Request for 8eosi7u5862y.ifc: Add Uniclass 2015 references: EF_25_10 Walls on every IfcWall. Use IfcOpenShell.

First a look at what the model holds.

```python
import ifcopenshell

model = ifcopenshell.open("8eosi7u5862y.ifc")
print(model.schema)
print("classifications:", [c.Name for c in model.by_type("IfcClassification")])
for ifc_class in ("IfcDoor", "IfcRoof", "IfcStair", "IfcWall", "IfcWindow"):
    print(ifc_class, len(model.by_type(ifc_class)))
```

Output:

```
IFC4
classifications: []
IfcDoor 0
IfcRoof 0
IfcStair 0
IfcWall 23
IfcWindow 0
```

```python
import ifcopenshell
import ifcopenshell.api.classification

model = ifcopenshell.open("8eosi7u5862y.ifc")

system = ifcopenshell.api.classification.add_classification(model, classification="Uniclass 2015")

codes = {
    "IfcWall": ("EF_25_10", "Walls"),
}
for ifc_class, (code, name) in codes.items():
    products = model.by_type(ifc_class)
    ifcopenshell.api.classification.add_reference(
        model, products=products, classification=system, identification=code, name=name
    )
    print(code, len(products))

model.write("8eosi7u5862y_updated.ifc")
```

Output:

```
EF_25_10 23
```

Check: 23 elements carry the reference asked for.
